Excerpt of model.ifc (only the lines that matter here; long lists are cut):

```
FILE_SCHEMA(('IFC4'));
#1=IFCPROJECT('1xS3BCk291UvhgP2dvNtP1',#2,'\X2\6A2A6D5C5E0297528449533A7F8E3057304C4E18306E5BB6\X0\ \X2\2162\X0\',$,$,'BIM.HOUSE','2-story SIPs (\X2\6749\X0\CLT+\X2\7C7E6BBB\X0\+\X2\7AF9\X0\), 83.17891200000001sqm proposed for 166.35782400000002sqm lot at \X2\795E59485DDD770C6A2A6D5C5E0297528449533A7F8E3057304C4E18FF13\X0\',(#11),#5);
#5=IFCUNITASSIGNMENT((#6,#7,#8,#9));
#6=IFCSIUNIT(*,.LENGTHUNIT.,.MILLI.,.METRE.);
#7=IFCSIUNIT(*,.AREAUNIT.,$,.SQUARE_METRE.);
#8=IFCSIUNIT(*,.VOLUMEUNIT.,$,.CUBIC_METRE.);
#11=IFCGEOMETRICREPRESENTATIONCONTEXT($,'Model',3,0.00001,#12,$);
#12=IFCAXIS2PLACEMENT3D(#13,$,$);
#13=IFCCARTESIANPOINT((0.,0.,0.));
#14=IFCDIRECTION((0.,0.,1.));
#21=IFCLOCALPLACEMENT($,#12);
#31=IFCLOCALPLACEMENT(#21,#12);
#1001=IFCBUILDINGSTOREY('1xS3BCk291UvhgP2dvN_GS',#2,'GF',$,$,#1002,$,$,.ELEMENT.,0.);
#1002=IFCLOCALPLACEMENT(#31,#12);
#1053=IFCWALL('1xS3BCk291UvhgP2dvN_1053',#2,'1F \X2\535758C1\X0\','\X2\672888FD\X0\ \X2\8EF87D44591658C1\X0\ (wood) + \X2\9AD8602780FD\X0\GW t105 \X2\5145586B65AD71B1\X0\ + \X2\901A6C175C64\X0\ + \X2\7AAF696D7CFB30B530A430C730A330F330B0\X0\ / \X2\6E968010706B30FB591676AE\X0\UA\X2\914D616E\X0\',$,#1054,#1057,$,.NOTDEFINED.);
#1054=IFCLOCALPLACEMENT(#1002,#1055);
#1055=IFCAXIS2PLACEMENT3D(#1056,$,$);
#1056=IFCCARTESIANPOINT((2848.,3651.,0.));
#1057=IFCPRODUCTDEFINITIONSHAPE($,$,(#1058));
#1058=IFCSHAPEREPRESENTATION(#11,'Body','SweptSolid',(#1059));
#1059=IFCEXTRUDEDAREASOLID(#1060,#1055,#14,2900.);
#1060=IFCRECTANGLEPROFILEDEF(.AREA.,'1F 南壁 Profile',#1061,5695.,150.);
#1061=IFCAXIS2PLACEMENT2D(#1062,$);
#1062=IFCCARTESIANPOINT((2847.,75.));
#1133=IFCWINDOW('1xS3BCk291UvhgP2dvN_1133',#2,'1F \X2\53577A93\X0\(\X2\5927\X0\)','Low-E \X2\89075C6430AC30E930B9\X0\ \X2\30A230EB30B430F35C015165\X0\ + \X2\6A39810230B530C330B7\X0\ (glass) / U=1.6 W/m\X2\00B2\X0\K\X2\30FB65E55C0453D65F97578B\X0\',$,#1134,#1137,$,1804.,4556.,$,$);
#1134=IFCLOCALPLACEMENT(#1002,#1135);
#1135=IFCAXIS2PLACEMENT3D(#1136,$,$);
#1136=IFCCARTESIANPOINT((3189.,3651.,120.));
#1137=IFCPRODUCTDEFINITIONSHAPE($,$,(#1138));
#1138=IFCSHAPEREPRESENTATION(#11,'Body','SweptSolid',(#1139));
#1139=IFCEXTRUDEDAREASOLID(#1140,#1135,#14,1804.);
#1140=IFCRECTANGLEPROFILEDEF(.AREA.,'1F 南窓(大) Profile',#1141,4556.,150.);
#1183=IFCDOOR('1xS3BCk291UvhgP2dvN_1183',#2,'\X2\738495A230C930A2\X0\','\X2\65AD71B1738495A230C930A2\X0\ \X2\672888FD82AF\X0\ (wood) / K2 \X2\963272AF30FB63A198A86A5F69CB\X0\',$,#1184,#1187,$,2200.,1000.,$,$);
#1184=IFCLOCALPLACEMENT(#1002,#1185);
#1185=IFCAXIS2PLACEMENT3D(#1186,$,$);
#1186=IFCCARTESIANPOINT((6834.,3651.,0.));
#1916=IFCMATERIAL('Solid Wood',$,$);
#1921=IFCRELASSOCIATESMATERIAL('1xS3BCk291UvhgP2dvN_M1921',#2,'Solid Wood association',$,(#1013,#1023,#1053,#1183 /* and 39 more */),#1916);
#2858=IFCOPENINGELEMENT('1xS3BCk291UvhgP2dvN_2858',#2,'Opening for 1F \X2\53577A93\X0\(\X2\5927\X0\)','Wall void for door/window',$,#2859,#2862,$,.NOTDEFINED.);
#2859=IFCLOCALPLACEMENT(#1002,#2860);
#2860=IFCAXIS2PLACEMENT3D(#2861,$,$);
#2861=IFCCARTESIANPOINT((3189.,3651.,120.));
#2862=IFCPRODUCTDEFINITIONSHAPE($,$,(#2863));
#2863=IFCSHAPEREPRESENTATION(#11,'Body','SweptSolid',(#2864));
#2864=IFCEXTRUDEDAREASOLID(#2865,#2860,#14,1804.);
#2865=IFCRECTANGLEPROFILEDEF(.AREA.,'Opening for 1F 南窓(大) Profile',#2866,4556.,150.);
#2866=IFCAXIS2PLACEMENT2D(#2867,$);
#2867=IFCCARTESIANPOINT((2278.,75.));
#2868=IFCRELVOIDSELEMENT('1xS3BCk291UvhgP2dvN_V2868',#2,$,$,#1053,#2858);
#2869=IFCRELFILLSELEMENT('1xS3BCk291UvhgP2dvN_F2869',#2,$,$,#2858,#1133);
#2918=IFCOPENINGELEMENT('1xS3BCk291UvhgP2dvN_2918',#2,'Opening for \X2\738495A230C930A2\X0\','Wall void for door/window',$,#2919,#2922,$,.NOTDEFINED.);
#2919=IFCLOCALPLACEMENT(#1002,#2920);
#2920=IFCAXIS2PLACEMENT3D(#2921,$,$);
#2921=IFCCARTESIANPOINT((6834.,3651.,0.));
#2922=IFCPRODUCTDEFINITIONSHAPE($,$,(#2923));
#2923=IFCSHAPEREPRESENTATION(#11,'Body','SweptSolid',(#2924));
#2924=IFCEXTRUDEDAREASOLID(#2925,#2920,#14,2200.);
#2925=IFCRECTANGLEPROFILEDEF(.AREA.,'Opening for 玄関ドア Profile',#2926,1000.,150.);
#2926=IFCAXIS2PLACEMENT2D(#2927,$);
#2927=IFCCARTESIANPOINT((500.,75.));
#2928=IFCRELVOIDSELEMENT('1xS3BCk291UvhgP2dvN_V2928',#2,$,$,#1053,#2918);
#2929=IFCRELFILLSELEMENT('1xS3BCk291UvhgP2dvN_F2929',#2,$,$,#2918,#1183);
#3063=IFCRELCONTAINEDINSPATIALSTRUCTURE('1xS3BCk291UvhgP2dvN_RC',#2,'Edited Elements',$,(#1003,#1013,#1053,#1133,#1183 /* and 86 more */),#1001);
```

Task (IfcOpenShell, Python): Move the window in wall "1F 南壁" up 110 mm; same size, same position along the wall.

```python
import numpy as np
import ifcopenshell
import ifcopenshell.api.geometry
import ifcopenshell.util.placement
import ifcopenshell.util.unit

model = ifcopenshell.open("model.ifc")
unit_scale = ifcopenshell.util.unit.calculate_unit_scale(model)

window = model.by_id(1133)
opening = window.FillsVoids[0].RelatingOpeningElement
dz = 110.0

shift = np.array([0.0, 0.0, dz])
# The window is not placed relative to its opening, so move both.
for product in (opening, window):
    matrix = ifcopenshell.util.placement.get_local_placement(product.ObjectPlacement)
    matrix[:3, 3] += shift
    ifcopenshell.api.geometry.edit_object_placement(model, product=product, matrix=matrix, is_si=False)

print(f"moved by {dz * unit_scale:+.3f} m")

model.write("model_v2.ifc")
```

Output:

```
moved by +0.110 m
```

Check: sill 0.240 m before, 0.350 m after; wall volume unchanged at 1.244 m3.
